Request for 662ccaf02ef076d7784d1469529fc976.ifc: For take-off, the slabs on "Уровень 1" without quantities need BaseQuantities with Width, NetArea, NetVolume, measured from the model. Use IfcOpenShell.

First a look at what the model holds.

```python
import ifcopenshell
import ifcopenshell.util.element
import ifcopenshell.util.unit

model = ifcopenshell.open("662ccaf02ef076d7784d1469529fc976.ifc")
print(model.schema)
for unit_type in ("LENGTHUNIT", "AREAUNIT", "VOLUMEUNIT"):
    print(unit_type, ifcopenshell.util.unit.calculate_unit_scale(model, unit_type))
storey = next(s for s in model.by_type("IfcBuildingStorey") if s.Name == "Уровень 1")
slabs = [e for e in ifcopenshell.util.element.get_decomposition(storey) if e.is_a("IfcSlab")]
for e in sorted(slabs, key=lambda e: e.id()):
    print(e.id(), e.is_a(), e.Name, list(ifcopenshell.util.element.get_psets(e, qtos_only=True)), sep=" | ")
```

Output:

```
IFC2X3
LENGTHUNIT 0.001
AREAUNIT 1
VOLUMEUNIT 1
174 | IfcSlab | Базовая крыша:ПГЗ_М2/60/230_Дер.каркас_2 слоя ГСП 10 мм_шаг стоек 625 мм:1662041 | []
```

```python
import ifcopenshell
import ifcopenshell.api.pset
import ifcopenshell.geom
import ifcopenshell.util.element
import ifcopenshell.util.shape
import ifcopenshell.util.unit

model = ifcopenshell.open("662ccaf02ef076d7784d1469529fc976.ifc")
unit_scale = ifcopenshell.util.unit.calculate_unit_scale(model)
area_scale = ifcopenshell.util.unit.calculate_unit_scale(model, "AREAUNIT")
volume_scale = ifcopenshell.util.unit.calculate_unit_scale(model, "VOLUMEUNIT")
settings = ifcopenshell.geom.settings()

storey = next(s for s in model.by_type("IfcBuildingStorey") if s.Name == "Уровень 1")
slabs = [e for e in ifcopenshell.util.element.get_decomposition(storey) if e.is_a("IfcSlab")]

for e in sorted(slabs, key=lambda e: e.id()):
    if ifcopenshell.util.element.get_psets(e, qtos_only=True, should_inherit=False):
        continue
    # Geometry comes back in metres, in the element's own axes.
    shape = ifcopenshell.geom.create_shape(settings, e)
    values = {
        "Width": ifcopenshell.util.shape.get_z(shape.geometry) / unit_scale,
        "NetArea": ifcopenshell.util.shape.get_footprint_area(shape.geometry) / area_scale,
        "NetVolume": ifcopenshell.util.shape.get_volume(shape.geometry) / volume_scale,
    }
    qto = ifcopenshell.api.pset.add_qto(model, product=e, name="BaseQuantities")
    ifcopenshell.api.pset.edit_qto(model, qto=qto, properties=values)
    print(e.id(), {k: round(v, 3) for k, v in values.items()})

model.write("662ccaf02ef076d7784d1469529fc976_rev.ifc")
```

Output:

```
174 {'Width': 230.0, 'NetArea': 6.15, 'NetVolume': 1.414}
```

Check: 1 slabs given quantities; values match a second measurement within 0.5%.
